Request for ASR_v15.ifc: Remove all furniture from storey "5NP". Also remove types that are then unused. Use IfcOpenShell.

First a look at what the model holds.

```python
import ifcopenshell
import ifcopenshell.util.element

model = ifcopenshell.open("ASR_v15.ifc")
print(model.schema)
storey = next(s for s in model.by_type("IfcBuildingStorey") if s.Name == "5NP")
furniture = [e for e in ifcopenshell.util.element.get_decomposition(storey) if e.is_a("IfcFurnishingElement")]
seen = {}
for e in furniture:
    element_type = ifcopenshell.util.element.get_type(e)
    name = element_type.Name if element_type not in (None, e) else None
    seen[name] = seen.get(name, 0) + 1
for name, count in sorted(seen.items(), key=str):
    print(count, "x", name)
```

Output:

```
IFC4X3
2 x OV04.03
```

```python
import ifcopenshell
import ifcopenshell.api.root
import ifcopenshell.util.element

model = ifcopenshell.open("ASR_v15.ifc")

storey = next(s for s in model.by_type("IfcBuildingStorey") if s.Name == "5NP")
furniture = [e for e in ifcopenshell.util.element.get_decomposition(storey) if e.is_a("IfcFurnishingElement")]
types = {ifcopenshell.util.element.get_type(e) for e in furniture} - {None, *furniture}

for e in furniture:
    ifcopenshell.api.root.remove_product(model, product=e)
print(len(furniture), "removed")

unused = [t for t in types if not ifcopenshell.util.element.get_types(t)]
for t in unused:
    ifcopenshell.api.root.remove_product(model, product=t)
print(len(unused), "unused types removed")

model.write("ASR_v15_v2.ifc")
```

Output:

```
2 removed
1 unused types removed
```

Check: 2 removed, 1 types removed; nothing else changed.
